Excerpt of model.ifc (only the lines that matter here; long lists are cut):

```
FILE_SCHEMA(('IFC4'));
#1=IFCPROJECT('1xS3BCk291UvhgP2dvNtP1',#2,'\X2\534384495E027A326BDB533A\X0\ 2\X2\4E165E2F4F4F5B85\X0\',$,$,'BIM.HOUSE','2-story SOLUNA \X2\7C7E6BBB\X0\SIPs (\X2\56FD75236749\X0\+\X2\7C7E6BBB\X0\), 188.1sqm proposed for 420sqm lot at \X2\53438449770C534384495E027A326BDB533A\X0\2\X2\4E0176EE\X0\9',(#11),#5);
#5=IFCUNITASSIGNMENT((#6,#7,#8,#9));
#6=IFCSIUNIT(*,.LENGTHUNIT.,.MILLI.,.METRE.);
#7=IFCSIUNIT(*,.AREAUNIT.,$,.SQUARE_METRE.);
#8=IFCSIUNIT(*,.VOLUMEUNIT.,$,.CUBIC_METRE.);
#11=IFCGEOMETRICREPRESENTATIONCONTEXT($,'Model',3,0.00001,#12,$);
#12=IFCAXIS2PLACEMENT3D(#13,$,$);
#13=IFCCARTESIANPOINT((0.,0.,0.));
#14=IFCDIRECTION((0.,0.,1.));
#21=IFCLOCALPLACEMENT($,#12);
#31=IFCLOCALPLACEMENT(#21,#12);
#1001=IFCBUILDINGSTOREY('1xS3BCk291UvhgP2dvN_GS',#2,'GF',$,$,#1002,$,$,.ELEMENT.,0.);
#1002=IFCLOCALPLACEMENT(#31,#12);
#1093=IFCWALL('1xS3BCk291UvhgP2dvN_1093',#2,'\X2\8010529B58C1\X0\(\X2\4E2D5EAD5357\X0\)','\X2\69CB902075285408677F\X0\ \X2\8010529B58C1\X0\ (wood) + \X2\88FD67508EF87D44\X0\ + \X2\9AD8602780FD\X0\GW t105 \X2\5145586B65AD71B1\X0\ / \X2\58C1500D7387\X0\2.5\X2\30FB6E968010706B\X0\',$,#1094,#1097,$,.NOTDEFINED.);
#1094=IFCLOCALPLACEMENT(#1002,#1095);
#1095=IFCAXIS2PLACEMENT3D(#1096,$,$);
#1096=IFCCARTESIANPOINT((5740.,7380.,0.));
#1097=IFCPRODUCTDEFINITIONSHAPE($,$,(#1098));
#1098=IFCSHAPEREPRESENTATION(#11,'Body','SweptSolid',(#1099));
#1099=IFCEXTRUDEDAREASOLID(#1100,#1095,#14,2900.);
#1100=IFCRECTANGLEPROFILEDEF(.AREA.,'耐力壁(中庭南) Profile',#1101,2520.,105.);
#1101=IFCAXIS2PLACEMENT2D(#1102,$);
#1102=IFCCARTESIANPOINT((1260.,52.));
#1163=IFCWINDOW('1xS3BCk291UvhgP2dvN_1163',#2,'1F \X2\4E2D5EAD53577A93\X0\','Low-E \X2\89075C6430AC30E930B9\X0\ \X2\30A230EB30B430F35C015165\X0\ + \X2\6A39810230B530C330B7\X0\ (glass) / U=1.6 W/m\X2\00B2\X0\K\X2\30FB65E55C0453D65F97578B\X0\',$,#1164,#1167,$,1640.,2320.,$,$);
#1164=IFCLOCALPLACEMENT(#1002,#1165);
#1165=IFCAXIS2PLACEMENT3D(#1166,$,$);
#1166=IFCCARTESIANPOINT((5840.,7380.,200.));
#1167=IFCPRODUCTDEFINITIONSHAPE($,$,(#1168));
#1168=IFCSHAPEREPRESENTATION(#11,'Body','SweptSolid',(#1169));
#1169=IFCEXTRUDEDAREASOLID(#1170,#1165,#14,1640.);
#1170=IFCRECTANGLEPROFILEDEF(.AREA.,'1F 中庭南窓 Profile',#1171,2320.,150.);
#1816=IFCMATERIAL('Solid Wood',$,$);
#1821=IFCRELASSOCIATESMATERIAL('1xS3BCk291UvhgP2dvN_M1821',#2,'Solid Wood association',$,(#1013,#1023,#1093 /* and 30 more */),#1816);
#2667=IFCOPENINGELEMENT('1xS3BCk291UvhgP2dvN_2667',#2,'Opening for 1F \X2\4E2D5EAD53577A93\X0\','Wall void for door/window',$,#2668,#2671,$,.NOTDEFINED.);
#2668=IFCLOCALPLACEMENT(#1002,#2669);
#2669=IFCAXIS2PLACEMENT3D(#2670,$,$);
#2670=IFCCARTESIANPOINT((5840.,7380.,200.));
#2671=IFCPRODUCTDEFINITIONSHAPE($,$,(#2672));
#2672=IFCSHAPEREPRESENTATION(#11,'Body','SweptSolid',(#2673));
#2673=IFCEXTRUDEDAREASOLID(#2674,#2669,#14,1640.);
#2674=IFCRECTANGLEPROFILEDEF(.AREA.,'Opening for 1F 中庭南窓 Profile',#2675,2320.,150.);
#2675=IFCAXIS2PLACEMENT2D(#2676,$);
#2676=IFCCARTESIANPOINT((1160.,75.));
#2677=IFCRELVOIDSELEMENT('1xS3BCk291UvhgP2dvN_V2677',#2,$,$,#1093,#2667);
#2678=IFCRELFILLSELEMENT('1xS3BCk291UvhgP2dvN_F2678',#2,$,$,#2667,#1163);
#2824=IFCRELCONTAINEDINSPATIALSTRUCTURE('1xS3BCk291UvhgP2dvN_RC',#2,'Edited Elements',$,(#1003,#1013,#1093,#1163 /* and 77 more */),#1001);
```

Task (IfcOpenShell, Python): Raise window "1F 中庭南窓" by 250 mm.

```python
import numpy as np
import ifcopenshell
import ifcopenshell.api.geometry
import ifcopenshell.util.placement
import ifcopenshell.util.unit

model = ifcopenshell.open("model.ifc")
unit_scale = ifcopenshell.util.unit.calculate_unit_scale(model)

window = model.by_guid("1xS3BCk291UvhgP2dvN_1163")
opening = window.FillsVoids[0].RelatingOpeningElement
dz = 0.25 / unit_scale

shift = np.array([0.0, 0.0, dz])
# The window is not placed relative to its opening, so move both.
for product in (opening, window):
    matrix = ifcopenshell.util.placement.get_local_placement(product.ObjectPlacement)
    matrix[:3, 3] += shift
    ifcopenshell.api.geometry.edit_object_placement(model, product=product, matrix=matrix, is_si=False)

print(f"moved by {dz * unit_scale:+.3f} m")

model.write("model-out.ifc")
```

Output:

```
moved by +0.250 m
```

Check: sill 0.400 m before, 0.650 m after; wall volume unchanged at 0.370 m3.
